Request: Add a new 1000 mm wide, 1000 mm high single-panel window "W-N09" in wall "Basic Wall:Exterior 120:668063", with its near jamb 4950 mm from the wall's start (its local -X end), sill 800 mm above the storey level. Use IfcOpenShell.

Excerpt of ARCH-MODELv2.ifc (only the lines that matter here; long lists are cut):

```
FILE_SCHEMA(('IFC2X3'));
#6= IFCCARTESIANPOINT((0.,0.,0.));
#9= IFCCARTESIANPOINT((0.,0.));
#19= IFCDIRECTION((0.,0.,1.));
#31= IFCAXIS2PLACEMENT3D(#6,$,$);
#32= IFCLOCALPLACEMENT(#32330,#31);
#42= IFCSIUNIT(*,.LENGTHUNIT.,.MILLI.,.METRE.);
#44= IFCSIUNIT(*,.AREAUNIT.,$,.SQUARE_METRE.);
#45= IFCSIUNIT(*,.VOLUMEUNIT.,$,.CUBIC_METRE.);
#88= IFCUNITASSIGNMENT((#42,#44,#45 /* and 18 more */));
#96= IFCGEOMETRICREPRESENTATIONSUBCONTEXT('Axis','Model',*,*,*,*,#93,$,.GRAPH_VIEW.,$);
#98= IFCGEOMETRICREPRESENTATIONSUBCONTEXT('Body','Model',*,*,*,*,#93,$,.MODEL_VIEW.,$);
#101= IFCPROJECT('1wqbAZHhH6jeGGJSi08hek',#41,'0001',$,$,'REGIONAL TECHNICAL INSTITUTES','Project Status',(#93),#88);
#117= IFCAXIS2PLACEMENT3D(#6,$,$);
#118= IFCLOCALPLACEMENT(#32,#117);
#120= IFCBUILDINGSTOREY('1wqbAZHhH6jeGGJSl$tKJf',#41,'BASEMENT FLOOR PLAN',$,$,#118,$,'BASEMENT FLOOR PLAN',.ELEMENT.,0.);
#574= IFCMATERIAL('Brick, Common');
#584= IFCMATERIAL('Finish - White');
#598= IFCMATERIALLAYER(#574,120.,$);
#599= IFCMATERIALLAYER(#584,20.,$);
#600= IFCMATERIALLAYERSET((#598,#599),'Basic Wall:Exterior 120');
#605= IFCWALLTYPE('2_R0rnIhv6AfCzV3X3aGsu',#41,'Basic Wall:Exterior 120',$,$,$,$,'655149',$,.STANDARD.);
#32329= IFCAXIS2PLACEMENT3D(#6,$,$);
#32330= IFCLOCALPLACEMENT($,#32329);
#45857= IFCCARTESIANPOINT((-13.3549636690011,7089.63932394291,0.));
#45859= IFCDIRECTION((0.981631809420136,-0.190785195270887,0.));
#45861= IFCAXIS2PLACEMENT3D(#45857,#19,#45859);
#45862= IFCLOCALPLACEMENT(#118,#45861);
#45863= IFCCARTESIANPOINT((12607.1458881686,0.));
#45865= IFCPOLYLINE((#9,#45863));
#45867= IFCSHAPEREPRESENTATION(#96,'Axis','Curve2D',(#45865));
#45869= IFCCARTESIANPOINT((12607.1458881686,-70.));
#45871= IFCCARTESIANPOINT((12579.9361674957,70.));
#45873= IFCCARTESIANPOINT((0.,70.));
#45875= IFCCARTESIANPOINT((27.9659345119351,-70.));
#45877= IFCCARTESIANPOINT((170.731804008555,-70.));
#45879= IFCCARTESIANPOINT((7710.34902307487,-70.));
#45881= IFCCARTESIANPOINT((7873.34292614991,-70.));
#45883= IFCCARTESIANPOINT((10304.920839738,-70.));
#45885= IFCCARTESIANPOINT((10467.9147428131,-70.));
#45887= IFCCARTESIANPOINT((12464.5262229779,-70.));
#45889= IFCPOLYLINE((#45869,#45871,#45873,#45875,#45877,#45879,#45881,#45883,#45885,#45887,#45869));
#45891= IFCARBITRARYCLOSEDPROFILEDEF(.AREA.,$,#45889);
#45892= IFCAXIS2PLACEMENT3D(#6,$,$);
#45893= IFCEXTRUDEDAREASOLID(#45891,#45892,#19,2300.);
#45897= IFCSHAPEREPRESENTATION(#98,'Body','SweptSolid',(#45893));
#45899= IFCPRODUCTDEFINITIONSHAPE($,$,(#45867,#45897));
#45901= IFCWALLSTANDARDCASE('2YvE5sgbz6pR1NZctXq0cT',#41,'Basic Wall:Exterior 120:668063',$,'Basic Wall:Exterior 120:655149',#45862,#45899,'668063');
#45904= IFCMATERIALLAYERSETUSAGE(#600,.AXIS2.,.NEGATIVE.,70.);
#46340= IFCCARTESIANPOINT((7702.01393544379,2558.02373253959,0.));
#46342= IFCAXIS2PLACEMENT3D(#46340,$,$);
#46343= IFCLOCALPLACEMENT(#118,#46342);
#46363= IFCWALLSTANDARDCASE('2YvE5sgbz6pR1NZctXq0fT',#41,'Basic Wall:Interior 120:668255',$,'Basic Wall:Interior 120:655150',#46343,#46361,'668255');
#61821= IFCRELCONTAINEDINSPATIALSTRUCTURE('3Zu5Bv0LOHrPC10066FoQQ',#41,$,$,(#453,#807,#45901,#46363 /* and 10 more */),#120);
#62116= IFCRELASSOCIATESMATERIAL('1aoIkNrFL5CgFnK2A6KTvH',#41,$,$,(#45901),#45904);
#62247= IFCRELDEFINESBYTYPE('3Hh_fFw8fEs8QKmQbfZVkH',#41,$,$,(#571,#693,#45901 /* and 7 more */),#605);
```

```python
import numpy as np
import ifcopenshell
import ifcopenshell.api.feature
import ifcopenshell.api.geometry
import ifcopenshell.api.root
import ifcopenshell.api.spatial
import ifcopenshell.api.type
import ifcopenshell.geom
import ifcopenshell.util.element
import ifcopenshell.util.placement
import ifcopenshell.util.representation
import ifcopenshell.util.shape
import ifcopenshell.util.unit

model = ifcopenshell.open("ARCH-MODELv2.ifc")
unit_scale = ifcopenshell.util.unit.calculate_unit_scale(model)
settings = ifcopenshell.geom.settings()


def volume(element):
    """Net volume in cubic metres, openings subtracted."""
    shape = ifcopenshell.geom.create_shape(settings, element)
    return ifcopenshell.util.shape.get_volume(shape.geometry)


wall = model.by_guid("2YvE5sgbz6pR1NZctXq0cT")
storey = ifcopenshell.util.element.get_container(wall, ifc_class="IfcBuildingStorey")
context = ifcopenshell.util.representation.get_context(model, "Model", "Body", "MODEL_VIEW")
before = volume(wall)

width, height, from_end, sill = 1, 1, 4.95, 0.8  # metres

# The wall runs along its own X axis, and the end named is its -X end.
wall_shape = ifcopenshell.geom.create_shape(settings, wall)
x, y, z = ifcopenshell.util.shape.get_vertices(wall_shape.geometry).T
start = x.min() + from_end
face, thickness = float(y.min()), float(y.max() - y.min())
wall_matrix = ifcopenshell.util.placement.get_local_placement(wall.ObjectPlacement)
level = ifcopenshell.util.placement.get_local_placement(storey.ObjectPlacement)[2, 3]


def in_wall(x, y):
    """Placement at x, y metres in the wall's axes, at sill height."""
    matrix = wall_matrix.copy()
    matrix[:, 3] = wall_matrix @ np.array([x / unit_scale, y / unit_scale, 0.0, 1.0])
    matrix[2, 3] = level + sill / unit_scale
    return matrix


# Opening: a box that overshoots both wall faces by 50 mm.
opening = ifcopenshell.api.root.create_entity(model, ifc_class="IfcOpeningElement")
box = ifcopenshell.api.geometry.add_wall_representation(
    model, context=context, length=width, height=height, thickness=thickness + 0.1
)
ifcopenshell.api.geometry.assign_representation(model, product=opening, representation=box)
ifcopenshell.api.geometry.edit_object_placement(model, product=opening, matrix=in_wall(start, face - 0.05), is_si=False)
ifcopenshell.api.feature.add_feature(model, feature=opening, element=wall)

window = ifcopenshell.api.root.create_entity(model, ifc_class="IfcWindow", name="W-N09")
window.OverallWidth, window.OverallHeight = width / unit_scale, height / unit_scale
body = ifcopenshell.api.geometry.add_window_representation(
    model,
    context=context,
    overall_width=window.OverallWidth,
    overall_height=window.OverallHeight,
    partition_type="SINGLE_PANEL",
)
ifcopenshell.api.geometry.assign_representation(model, product=window, representation=body)
ifcopenshell.api.spatial.assign_container(model, products=[window], relating_structure=storey)
fills = ifcopenshell.api.feature.add_filling(model, opening=opening, element=window)
fills.OwnerHistory = window.OwnerHistory  # required in IFC2X3

# IFC2X3 keeps the operation on the window style.
style = ifcopenshell.api.root.create_entity(model, ifc_class="IfcWindowStyle", name="W-N09")
style.OperationType, style.ConstructionType = "SINGLE_PANEL", "NOTDEFINED"
style.ParameterTakesPrecedence = style.Sizeable = False
ifcopenshell.api.type.assign_type(model, related_objects=[window], relating_type=style)

# Centre the window in the wall's thickness.
ifcopenshell.api.geometry.edit_object_placement(model, product=window, matrix=in_wall(start, face), is_si=False)
window_shape = ifcopenshell.geom.create_shape(settings, window)
depth = ifcopenshell.util.shape.get_vertices(window_shape.geometry)[:, 1]
offset = face + thickness / 2 - (depth.min() + depth.max()) / 2
ifcopenshell.api.geometry.edit_object_placement(model, product=window, matrix=in_wall(start, offset), is_si=False)

after = volume(wall)

print(f"wall volume {before:.3f} -> {after:.3f} m3")

model.write("ARCH-MODELv2_v2.ifc")
```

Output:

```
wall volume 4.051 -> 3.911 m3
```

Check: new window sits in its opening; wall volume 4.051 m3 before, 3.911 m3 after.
